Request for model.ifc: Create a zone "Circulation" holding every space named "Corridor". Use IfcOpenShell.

First a look at what the model holds.

```python
import ifcopenshell

model = ifcopenshell.open("model.ifc")
print(model.schema)
seen = {}
for space in model.by_type("IfcSpace"):
    seen[space.Name] = seen.get(space.Name, 0) + 1
for name, count in sorted(seen.items(), key=str):
    print(count, "x", name)
print("zones:", [z.Name for z in model.by_type("IfcZone")][:20])
```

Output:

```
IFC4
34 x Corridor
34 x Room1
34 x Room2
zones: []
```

```python
import ifcopenshell
import ifcopenshell.api.group
import ifcopenshell.api.root

model = ifcopenshell.open("model.ifc")

names = {"Corridor"}
spaces = [s for s in model.by_type("IfcSpace") if s.Name in names]

zone = ifcopenshell.api.root.create_entity(model, ifc_class="IfcZone", name="Circulation")
ifcopenshell.api.group.assign_group(model, products=spaces, group=zone)
print(len(spaces), "spaces in", zone.Name)

model.write("model_updated.ifc")
```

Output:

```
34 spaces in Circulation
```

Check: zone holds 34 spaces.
